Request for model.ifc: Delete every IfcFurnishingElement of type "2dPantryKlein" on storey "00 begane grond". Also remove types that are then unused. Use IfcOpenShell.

First a look at what the model holds.

```python
import ifcopenshell
import ifcopenshell.util.element

model = ifcopenshell.open("model.ifc")
print(model.schema)
storey = next(s for s in model.by_type("IfcBuildingStorey") if s.Name == "00 begane grond")
furniture = [e for e in ifcopenshell.util.element.get_decomposition(storey) if e.is_a("IfcFurnishingElement")]
seen = {}
for e in furniture:
    element_type = ifcopenshell.util.element.get_type(e)
    name = element_type.Name if element_type not in (None, e) else None
    seen[name] = seen.get(name, 0) + 1
for name, count in sorted(seen.items(), key=str):
    print(count, "x", name)
```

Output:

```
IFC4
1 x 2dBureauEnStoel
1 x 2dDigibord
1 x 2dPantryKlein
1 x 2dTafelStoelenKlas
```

```python
import ifcopenshell
import ifcopenshell.api.root
import ifcopenshell.util.element

model = ifcopenshell.open("model.ifc")

storey = next(s for s in model.by_type("IfcBuildingStorey") if s.Name == "00 begane grond")
furniture = [e for e in ifcopenshell.util.element.get_decomposition(storey) if e.is_a("IfcFurnishingElement")]
targets = [e for e in furniture if (t := ifcopenshell.util.element.get_type(e)) not in (None, e) and t.Name == "2dPantryKlein"]
types = {ifcopenshell.util.element.get_type(e) for e in targets} - {None, *targets}

for e in targets:
    ifcopenshell.api.root.remove_product(model, product=e)
print(len(targets), "removed")

unused = [t for t in types if not ifcopenshell.util.element.get_types(t)]
for t in unused:
    ifcopenshell.api.root.remove_product(model, product=t)
print(len(unused), "unused types removed")

model.write("model-out.ifc")
```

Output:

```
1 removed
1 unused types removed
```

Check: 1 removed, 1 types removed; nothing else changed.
